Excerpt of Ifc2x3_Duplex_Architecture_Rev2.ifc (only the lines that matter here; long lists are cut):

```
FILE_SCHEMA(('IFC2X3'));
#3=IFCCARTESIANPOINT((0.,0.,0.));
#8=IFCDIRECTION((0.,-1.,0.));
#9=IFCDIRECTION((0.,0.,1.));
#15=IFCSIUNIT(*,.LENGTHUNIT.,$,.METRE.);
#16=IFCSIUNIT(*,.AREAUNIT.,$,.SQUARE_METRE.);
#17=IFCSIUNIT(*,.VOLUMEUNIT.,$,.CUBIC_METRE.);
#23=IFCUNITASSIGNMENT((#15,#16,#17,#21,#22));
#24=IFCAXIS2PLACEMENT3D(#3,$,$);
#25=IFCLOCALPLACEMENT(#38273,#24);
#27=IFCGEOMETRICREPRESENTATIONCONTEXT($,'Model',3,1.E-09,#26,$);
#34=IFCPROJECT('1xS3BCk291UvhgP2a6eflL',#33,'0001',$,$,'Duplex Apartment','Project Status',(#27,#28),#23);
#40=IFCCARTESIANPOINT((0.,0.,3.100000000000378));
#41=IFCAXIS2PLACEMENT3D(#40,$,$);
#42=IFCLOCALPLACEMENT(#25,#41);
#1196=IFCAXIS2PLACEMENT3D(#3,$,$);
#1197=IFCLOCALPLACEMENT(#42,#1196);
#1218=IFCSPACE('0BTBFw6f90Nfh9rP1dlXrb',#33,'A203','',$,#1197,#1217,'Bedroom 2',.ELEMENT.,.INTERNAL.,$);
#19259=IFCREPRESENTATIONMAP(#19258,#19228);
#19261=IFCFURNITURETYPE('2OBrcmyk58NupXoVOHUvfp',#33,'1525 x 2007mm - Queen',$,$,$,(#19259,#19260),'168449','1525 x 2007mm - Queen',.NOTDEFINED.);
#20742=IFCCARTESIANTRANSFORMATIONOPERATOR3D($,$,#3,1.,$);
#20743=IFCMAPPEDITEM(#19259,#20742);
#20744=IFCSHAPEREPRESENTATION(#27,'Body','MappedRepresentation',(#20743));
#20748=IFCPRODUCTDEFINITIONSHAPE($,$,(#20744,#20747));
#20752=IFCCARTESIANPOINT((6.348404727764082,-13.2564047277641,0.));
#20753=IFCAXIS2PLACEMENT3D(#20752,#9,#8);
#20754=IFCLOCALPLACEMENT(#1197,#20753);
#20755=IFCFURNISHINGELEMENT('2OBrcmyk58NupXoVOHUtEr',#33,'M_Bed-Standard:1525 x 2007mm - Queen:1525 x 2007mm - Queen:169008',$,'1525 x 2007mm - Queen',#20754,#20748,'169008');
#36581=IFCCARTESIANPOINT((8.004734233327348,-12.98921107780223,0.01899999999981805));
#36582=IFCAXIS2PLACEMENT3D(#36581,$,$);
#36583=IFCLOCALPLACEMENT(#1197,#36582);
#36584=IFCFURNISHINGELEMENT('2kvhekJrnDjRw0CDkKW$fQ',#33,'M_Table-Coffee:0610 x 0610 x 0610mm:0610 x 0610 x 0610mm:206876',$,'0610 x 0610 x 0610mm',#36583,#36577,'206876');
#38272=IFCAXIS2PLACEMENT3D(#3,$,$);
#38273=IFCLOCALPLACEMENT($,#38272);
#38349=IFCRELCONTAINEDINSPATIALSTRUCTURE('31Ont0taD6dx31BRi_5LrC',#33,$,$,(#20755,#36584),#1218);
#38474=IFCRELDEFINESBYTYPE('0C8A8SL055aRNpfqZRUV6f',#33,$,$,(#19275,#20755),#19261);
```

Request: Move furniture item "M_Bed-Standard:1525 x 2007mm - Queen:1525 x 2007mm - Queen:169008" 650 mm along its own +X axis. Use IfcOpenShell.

```python
import ifcopenshell
import ifcopenshell.api.geometry
import ifcopenshell.util.placement
import ifcopenshell.util.unit

model = ifcopenshell.open("Ifc2x3_Duplex_Architecture_Rev2.ifc")
unit_scale = ifcopenshell.util.unit.calculate_unit_scale(model)

item = model.by_guid("2OBrcmyk58NupXoVOHUtEr")
matrix = ifcopenshell.util.placement.get_local_placement(item.ObjectPlacement)
matrix[:3, 3] += matrix[:3, 0] * 0.65 / unit_scale
ifcopenshell.api.geometry.edit_object_placement(model, product=item, matrix=matrix, is_si=False)

print(ifcopenshell.util.placement.get_local_placement(item.ObjectPlacement).round(3) + 0.0)

model.write("Ifc2x3_Duplex_Architecture_Rev2_edited.ifc")
```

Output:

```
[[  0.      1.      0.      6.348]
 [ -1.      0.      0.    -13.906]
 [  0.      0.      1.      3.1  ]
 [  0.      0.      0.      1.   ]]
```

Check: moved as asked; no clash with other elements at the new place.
